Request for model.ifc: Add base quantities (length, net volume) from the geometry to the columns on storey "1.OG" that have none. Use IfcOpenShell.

First a look at what the model holds.

```python
import ifcopenshell
import ifcopenshell.util.element
import ifcopenshell.util.unit

model = ifcopenshell.open("model.ifc")
print(model.schema)
for unit_type in ("LENGTHUNIT", "AREAUNIT", "VOLUMEUNIT"):
    print(unit_type, ifcopenshell.util.unit.calculate_unit_scale(model, unit_type))
storey = next(s for s in model.by_type("IfcBuildingStorey") if s.Name == "1.OG")
columns = [e for e in ifcopenshell.util.element.get_decomposition(storey) if e.is_a("IfcColumn")]
for e in sorted(columns, key=lambda e: e.id()):
    print(e.id(), e.is_a(), e.Name, list(ifcopenshell.util.element.get_psets(e, qtos_only=True)), sep=" | ")
```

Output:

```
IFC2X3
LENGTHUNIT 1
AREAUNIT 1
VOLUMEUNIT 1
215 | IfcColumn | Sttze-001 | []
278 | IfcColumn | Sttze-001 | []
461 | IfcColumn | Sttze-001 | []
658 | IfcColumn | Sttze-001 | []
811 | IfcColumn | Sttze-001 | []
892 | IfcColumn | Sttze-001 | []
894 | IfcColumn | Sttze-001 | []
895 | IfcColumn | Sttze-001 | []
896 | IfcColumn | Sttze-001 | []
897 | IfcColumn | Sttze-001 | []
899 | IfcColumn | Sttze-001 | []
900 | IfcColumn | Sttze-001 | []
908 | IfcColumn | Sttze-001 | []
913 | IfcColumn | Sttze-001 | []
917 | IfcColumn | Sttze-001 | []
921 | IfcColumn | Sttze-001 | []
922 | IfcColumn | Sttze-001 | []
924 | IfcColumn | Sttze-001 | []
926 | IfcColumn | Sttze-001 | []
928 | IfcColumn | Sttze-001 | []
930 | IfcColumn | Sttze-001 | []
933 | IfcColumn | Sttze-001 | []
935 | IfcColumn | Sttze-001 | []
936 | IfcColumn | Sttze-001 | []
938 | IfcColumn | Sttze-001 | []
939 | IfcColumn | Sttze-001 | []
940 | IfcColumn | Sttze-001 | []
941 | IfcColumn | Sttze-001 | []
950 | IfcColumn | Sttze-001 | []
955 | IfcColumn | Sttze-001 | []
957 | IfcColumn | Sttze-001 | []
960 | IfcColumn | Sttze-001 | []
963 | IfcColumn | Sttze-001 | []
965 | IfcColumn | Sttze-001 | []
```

```python
import ifcopenshell
import ifcopenshell.api.pset
import ifcopenshell.geom
import ifcopenshell.util.element
import ifcopenshell.util.shape
import ifcopenshell.util.unit

model = ifcopenshell.open("model.ifc")
unit_scale = ifcopenshell.util.unit.calculate_unit_scale(model)
volume_scale = ifcopenshell.util.unit.calculate_unit_scale(model, "VOLUMEUNIT")
settings = ifcopenshell.geom.settings()

storey = next(s for s in model.by_type("IfcBuildingStorey") if s.Name == "1.OG")
columns = [e for e in ifcopenshell.util.element.get_decomposition(storey) if e.is_a("IfcColumn")]

for e in sorted(columns, key=lambda e: e.id()):
    if ifcopenshell.util.element.get_psets(e, qtos_only=True, should_inherit=False):
        continue
    # Geometry comes back in metres, in the element's own axes.
    shape = ifcopenshell.geom.create_shape(settings, e)
    values = {
        "Length": ifcopenshell.util.shape.get_z(shape.geometry) / unit_scale,
        "NetVolume": ifcopenshell.util.shape.get_volume(shape.geometry) / volume_scale,
    }
    qto = ifcopenshell.api.pset.add_qto(model, product=e, name="BaseQuantities")
    ifcopenshell.api.pset.edit_qto(model, qto=qto, properties=values)
    print(e.id(), {k: round(v, 3) for k, v in values.items()})

model.write("model_v2.ifc")
```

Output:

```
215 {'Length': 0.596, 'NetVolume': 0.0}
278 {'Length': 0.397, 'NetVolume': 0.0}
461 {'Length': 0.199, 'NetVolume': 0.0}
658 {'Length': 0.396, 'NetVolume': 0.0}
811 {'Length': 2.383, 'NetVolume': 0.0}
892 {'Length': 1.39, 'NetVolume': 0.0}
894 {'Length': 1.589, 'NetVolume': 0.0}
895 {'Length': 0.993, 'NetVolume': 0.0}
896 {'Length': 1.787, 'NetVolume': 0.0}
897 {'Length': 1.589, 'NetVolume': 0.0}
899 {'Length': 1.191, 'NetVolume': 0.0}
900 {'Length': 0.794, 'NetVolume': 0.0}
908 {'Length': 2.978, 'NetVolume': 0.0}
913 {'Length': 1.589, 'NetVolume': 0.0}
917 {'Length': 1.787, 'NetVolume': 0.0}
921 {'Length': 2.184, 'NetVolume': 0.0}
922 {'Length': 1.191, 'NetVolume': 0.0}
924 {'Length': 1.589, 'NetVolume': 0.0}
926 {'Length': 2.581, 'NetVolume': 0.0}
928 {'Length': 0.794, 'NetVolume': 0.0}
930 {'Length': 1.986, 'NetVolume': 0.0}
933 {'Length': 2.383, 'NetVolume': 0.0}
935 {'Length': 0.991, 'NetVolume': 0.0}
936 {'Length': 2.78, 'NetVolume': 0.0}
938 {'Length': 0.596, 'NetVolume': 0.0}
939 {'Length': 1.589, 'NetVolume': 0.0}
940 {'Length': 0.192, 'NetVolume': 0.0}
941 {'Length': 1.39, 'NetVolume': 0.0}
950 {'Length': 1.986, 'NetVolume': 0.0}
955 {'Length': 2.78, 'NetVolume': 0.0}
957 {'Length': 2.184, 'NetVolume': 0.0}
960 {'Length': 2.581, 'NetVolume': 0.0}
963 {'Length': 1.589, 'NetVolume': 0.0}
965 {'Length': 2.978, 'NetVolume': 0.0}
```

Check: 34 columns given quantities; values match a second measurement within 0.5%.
